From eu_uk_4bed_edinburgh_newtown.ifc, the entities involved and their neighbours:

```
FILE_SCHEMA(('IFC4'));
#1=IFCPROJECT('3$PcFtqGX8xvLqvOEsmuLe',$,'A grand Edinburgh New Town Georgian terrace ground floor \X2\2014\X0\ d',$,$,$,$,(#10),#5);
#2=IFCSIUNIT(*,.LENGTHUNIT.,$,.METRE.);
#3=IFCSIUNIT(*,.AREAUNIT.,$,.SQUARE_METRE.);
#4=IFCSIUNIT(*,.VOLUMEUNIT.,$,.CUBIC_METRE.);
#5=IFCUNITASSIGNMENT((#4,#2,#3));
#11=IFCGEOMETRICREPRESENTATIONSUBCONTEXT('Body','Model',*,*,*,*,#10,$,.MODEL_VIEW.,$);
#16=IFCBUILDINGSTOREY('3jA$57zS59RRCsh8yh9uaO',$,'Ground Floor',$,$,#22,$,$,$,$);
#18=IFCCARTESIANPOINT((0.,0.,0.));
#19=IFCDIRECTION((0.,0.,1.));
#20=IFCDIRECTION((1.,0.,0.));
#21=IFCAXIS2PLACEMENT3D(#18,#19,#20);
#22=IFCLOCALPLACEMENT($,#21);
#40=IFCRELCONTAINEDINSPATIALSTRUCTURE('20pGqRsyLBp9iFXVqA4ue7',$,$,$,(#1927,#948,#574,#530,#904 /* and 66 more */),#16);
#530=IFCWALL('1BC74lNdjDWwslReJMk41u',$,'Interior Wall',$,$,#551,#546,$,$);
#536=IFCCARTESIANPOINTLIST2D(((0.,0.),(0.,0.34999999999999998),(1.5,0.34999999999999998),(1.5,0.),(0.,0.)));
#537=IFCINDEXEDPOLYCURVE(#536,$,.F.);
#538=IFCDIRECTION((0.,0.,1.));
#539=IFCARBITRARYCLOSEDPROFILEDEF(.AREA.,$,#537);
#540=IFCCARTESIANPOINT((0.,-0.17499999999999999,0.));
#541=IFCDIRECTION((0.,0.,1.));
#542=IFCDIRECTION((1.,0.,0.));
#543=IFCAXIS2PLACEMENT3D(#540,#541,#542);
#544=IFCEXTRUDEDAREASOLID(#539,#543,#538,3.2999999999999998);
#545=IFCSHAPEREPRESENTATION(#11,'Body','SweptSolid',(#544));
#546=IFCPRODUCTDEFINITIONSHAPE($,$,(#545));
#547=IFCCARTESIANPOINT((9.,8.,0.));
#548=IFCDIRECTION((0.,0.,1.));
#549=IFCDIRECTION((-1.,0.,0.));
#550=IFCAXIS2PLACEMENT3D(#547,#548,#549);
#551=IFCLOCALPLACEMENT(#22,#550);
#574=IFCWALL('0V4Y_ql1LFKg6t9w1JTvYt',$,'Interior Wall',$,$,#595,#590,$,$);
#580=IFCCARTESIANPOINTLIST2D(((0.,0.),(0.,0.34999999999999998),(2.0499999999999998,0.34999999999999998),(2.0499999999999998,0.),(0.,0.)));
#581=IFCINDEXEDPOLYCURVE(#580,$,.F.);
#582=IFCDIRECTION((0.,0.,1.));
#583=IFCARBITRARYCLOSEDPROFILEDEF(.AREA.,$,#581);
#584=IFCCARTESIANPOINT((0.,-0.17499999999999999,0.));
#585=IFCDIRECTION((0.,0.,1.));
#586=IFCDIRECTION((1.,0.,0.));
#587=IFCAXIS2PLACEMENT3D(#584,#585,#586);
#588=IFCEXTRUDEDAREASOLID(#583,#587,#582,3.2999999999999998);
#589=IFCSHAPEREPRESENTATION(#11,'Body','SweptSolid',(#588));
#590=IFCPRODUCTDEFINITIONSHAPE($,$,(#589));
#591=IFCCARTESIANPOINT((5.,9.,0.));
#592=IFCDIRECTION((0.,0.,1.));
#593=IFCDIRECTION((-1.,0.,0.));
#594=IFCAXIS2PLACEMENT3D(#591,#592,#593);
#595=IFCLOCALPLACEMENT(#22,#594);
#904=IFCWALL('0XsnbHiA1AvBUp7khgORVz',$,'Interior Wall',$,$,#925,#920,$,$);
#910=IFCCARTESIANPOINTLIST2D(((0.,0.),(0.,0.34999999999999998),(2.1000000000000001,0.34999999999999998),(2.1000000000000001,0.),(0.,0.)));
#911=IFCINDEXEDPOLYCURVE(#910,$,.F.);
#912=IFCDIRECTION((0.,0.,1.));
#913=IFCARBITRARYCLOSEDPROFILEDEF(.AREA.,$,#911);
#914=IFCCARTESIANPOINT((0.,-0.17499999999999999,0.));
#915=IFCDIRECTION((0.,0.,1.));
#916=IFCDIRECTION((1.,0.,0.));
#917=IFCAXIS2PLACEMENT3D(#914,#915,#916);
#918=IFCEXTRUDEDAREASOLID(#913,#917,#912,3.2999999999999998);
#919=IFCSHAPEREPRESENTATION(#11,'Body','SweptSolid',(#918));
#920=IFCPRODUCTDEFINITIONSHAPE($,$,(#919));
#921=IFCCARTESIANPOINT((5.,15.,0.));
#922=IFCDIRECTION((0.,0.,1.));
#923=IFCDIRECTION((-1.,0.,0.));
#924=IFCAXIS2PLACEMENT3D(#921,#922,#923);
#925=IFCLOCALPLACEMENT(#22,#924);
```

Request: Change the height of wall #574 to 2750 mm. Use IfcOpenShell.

```python
import ifcopenshell
import ifcopenshell.geom
import ifcopenshell.util.representation
import ifcopenshell.util.shape
import ifcopenshell.util.unit

model = ifcopenshell.open("eu_uk_4bed_edinburgh_newtown.ifc")
unit_scale = ifcopenshell.util.unit.calculate_unit_scale(model)
settings = ifcopenshell.geom.settings()


def volume(element):
    """Net volume in cubic metres, openings subtracted."""
    shape = ifcopenshell.geom.create_shape(settings, element)
    return ifcopenshell.util.shape.get_volume(shape.geometry)


wall = model.by_guid("0V4Y_ql1LFKg6t9w1JTvYt")
before = volume(wall)

body = ifcopenshell.util.representation.get_representation(wall, "Model", "Body")
solid = body.Items[0]
old_height = solid.Depth
solid.Depth = 2.75 / unit_scale
after = volume(wall)

print(f"height {old_height:g} -> {solid.Depth:g}, volume {before:.3f} -> {after:.3f} m3")

model.write("eu_uk_4bed_edinburgh_newtown-out.ifc")
```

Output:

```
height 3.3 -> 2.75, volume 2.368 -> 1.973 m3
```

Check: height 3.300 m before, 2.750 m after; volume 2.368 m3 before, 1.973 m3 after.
